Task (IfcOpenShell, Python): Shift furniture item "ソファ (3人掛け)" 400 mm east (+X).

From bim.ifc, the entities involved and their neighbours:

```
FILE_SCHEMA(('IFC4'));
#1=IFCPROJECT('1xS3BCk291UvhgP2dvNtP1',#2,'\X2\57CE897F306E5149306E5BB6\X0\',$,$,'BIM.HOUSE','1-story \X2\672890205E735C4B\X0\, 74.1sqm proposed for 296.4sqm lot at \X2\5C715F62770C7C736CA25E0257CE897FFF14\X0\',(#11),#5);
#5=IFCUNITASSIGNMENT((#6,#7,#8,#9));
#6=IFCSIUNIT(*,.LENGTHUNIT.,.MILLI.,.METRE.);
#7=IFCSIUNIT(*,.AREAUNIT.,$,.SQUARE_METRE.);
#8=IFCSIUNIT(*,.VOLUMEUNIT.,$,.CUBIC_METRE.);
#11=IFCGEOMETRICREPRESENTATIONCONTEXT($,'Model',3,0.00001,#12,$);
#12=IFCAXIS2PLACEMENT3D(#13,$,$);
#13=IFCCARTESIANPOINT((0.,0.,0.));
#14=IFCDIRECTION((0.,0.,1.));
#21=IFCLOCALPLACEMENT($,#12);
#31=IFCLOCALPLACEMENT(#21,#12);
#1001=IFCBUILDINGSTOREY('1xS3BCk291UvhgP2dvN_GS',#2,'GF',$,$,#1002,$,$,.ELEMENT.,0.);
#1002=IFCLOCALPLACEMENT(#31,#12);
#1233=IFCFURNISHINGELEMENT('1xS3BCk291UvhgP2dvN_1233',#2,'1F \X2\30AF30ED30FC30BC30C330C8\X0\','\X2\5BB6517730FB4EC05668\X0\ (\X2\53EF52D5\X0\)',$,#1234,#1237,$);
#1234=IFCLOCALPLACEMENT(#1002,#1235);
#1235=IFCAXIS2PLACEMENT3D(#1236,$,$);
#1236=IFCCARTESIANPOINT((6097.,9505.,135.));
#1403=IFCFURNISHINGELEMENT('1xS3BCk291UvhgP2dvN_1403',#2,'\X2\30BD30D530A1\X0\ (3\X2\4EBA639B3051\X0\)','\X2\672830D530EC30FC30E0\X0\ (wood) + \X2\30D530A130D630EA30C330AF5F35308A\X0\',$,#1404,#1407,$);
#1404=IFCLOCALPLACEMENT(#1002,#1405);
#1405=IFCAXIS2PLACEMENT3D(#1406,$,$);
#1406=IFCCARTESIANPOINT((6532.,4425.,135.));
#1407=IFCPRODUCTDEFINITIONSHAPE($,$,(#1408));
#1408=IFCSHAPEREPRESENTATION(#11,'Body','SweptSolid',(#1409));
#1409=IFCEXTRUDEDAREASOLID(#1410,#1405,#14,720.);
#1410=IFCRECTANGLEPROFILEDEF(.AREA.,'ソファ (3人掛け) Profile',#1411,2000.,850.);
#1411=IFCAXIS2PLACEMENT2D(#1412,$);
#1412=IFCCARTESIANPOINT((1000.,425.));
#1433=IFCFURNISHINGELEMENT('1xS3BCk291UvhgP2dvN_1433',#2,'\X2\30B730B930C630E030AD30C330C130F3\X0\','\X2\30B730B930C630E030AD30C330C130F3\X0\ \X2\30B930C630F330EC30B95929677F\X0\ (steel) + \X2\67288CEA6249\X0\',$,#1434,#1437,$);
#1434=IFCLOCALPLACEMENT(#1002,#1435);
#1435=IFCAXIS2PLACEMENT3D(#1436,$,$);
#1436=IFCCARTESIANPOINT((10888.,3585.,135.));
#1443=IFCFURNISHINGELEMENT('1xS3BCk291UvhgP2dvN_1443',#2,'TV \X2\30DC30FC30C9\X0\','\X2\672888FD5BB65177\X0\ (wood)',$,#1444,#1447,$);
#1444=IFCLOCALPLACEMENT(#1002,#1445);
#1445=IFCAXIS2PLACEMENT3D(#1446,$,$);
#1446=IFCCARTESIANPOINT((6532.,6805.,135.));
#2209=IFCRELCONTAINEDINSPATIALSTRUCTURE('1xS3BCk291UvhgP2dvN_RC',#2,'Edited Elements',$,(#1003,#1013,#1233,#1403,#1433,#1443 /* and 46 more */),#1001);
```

```python
import ifcopenshell
import ifcopenshell.api.geometry
import ifcopenshell.util.placement
import ifcopenshell.util.unit

model = ifcopenshell.open("bim.ifc")
unit_scale = ifcopenshell.util.unit.calculate_unit_scale(model)

item = model.by_id(1403)
matrix = ifcopenshell.util.placement.get_local_placement(item.ObjectPlacement)
matrix[0, 3] += 0.4 / unit_scale
ifcopenshell.api.geometry.edit_object_placement(model, product=item, matrix=matrix, is_si=False)

print(ifcopenshell.util.placement.get_local_placement(item.ObjectPlacement).round(3) + 0.0)

model.write("bim-out.ifc")
```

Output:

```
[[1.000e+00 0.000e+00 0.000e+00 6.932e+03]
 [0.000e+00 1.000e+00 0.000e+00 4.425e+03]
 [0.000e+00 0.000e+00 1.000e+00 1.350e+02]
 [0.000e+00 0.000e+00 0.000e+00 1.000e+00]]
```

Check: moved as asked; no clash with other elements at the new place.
